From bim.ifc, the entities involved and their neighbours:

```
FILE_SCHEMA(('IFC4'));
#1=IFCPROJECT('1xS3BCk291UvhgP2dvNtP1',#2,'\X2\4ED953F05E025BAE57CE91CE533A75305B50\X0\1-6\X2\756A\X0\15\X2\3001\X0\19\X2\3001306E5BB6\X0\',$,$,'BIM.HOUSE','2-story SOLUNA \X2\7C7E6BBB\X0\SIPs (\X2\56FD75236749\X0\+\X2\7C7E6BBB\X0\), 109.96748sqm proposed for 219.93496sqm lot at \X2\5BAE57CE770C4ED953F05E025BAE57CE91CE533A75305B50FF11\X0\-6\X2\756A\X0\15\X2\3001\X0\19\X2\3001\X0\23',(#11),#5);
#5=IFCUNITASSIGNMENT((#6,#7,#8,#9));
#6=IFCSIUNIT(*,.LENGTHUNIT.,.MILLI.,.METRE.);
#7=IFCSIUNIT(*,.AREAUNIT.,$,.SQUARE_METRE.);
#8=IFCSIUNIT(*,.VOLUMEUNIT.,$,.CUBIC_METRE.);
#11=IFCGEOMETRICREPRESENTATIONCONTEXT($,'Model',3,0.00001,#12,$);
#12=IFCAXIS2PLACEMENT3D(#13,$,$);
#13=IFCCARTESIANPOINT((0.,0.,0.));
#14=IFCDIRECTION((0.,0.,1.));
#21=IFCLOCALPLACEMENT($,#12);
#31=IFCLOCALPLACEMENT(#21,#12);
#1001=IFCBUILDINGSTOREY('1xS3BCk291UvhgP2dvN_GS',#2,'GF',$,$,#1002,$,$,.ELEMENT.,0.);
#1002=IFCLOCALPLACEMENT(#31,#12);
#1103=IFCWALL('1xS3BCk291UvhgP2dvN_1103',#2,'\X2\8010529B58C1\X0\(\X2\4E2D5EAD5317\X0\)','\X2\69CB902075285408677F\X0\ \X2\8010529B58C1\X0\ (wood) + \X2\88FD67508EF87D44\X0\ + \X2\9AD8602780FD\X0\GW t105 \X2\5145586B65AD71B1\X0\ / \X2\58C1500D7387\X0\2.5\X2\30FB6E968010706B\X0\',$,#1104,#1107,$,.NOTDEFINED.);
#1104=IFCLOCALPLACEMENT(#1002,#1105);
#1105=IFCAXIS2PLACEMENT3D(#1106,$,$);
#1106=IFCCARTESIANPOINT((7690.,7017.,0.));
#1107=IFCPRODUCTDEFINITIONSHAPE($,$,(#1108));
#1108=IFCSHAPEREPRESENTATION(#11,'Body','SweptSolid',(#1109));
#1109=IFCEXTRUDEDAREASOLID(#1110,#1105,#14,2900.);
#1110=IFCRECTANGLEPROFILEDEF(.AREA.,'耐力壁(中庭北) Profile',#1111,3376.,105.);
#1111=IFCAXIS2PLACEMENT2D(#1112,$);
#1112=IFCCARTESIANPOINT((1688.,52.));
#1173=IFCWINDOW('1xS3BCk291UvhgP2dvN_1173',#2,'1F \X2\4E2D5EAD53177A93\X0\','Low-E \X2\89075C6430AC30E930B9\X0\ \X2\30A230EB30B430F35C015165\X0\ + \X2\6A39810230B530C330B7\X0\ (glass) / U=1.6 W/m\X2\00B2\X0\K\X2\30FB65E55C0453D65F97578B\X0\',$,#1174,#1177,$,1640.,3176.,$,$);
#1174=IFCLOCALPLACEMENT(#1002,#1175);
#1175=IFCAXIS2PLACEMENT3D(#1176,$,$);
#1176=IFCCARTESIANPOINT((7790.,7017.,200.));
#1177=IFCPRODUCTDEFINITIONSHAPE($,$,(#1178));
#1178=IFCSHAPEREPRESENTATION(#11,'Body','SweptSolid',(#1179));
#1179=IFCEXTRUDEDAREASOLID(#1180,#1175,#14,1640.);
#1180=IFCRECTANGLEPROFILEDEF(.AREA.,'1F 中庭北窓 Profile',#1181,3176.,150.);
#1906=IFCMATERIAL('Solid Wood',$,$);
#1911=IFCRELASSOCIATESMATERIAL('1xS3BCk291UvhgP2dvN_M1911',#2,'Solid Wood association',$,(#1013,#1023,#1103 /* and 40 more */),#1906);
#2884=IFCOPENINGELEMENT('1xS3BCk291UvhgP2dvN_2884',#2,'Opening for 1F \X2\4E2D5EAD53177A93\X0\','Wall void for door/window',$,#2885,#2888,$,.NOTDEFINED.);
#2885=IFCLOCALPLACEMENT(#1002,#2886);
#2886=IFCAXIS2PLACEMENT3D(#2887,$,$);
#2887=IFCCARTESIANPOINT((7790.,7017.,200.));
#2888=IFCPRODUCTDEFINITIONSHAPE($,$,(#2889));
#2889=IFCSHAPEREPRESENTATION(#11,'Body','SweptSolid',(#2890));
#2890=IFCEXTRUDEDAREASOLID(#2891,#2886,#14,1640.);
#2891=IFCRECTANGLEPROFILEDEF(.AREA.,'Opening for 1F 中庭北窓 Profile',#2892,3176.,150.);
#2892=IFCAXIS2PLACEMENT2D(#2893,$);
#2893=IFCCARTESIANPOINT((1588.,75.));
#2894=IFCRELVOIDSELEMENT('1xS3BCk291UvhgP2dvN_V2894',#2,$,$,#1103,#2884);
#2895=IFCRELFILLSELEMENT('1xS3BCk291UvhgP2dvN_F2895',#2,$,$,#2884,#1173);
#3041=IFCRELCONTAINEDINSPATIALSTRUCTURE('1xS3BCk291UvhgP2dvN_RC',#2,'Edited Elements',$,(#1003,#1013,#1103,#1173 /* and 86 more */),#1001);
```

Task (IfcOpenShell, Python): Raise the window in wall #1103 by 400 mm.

```python
import numpy as np
import ifcopenshell
import ifcopenshell.api.geometry
import ifcopenshell.util.placement
import ifcopenshell.util.unit

model = ifcopenshell.open("bim.ifc")
unit_scale = ifcopenshell.util.unit.calculate_unit_scale(model)

window = model.by_guid("1xS3BCk291UvhgP2dvN_1173")
opening = window.FillsVoids[0].RelatingOpeningElement
dz = 0.4 / unit_scale

shift = np.array([0.0, 0.0, dz])
# The window is not placed relative to its opening, so move both.
for product in (opening, window):
    matrix = ifcopenshell.util.placement.get_local_placement(product.ObjectPlacement)
    matrix[:3, 3] += shift
    ifcopenshell.api.geometry.edit_object_placement(model, product=product, matrix=matrix, is_si=False)

print(f"moved by {dz * unit_scale:+.3f} m")

model.write("bim_edited.ifc")
```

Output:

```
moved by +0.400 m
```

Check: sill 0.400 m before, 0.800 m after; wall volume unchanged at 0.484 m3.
